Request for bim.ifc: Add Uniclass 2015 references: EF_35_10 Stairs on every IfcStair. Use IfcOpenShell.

First a look at what the model holds.

```python
import ifcopenshell

model = ifcopenshell.open("bim.ifc")
print(model.schema)
print("classifications:", [c.Name for c in model.by_type("IfcClassification")])
for ifc_class in ("IfcDoor", "IfcRoof", "IfcStair", "IfcWall", "IfcWindow"):
    print(ifc_class, len(model.by_type(ifc_class)))
```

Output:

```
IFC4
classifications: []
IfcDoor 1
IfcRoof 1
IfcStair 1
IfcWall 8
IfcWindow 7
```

```python
import ifcopenshell
import ifcopenshell.api.classification

model = ifcopenshell.open("bim.ifc")

system = ifcopenshell.api.classification.add_classification(model, classification="Uniclass 2015")

codes = {
    "IfcStair": ("EF_35_10", "Stairs"),
}
for ifc_class, (code, name) in codes.items():
    products = model.by_type(ifc_class)
    ifcopenshell.api.classification.add_reference(
        model, products=products, classification=system, identification=code, name=name
    )
    print(code, len(products))

model.write("bim_edited.ifc")
```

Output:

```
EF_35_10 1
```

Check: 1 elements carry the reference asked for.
